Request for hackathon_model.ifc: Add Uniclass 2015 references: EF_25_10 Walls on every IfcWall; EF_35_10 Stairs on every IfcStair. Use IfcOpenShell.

First a look at what the model holds.

```python
import ifcopenshell

model = ifcopenshell.open("hackathon_model.ifc")
print(model.schema)
print("classifications:", [c.Name for c in model.by_type("IfcClassification")])
for ifc_class in ("IfcDoor", "IfcRoof", "IfcStair", "IfcWall", "IfcWindow"):
    print(ifc_class, len(model.by_type(ifc_class)))
```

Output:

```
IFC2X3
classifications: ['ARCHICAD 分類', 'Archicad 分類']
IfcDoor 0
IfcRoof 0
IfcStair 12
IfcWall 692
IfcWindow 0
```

```python
import ifcopenshell
import ifcopenshell.api.classification

model = ifcopenshell.open("hackathon_model.ifc")

# IFC2X3 requires Source and Edition and has no link from the project to the system.
system = model.create_entity("IfcClassification", Source="NBS", Edition="2015", Name="Uniclass 2015")

codes = {
    "IfcWall": ("EF_25_10", "Walls"),
    "IfcStair": ("EF_35_10", "Stairs"),
}
for ifc_class, (code, name) in codes.items():
    products = model.by_type(ifc_class)
    ifcopenshell.api.classification.add_reference(
        model, products=products, classification=system, identification=code, name=name
    )
    print(code, len(products))

model.write("hackathon_model-out.ifc")
```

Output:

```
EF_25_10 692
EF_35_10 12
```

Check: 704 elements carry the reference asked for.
